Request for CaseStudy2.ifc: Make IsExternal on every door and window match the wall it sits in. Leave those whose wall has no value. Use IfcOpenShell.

First a look at what the model holds.

```python
import ifcopenshell
import ifcopenshell.util.element

model = ifcopenshell.open("CaseStudy2.ifc")
print(model.schema)
seen = {}
for e in model.by_type("IfcDoor") + model.by_type("IfcWindow"):
    if not e.FillsVoids:
        continue
    host = e.FillsVoids[0].RelatingOpeningElement.VoidsElements[0].RelatingBuildingElement
    own = ifcopenshell.util.element.get_pset(e, f"Pset_{e.is_a()[3:].removesuffix('StandardCase')}Common", "IsExternal")
    wall = ifcopenshell.util.element.get_pset(host, "Pset_WallCommon", "IsExternal")
    seen[e.is_a(), own, wall] = seen.get((e.is_a(), own, wall), 0) + 1
for (cls, own, wall), count in sorted(seen.items(), key=str):
    print(count, cls, "IsExternal:", own, "| host wall:", wall)
```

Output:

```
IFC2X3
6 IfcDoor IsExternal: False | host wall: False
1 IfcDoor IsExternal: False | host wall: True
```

```python
import ifcopenshell
import ifcopenshell.api.pset
import ifcopenshell.util.element

model = ifcopenshell.open("CaseStudy2.ifc")

count = 0
for ifc_class, pset_name in (("IfcDoor", "Pset_DoorCommon"), ("IfcWindow", "Pset_WindowCommon")):
    for e in model.by_type(ifc_class):
        if not e.FillsVoids:
            continue
        host = e.FillsVoids[0].RelatingOpeningElement.VoidsElements[0].RelatingBuildingElement
        external = ifcopenshell.util.element.get_pset(host, "Pset_WallCommon", "IsExternal")
        if external is None or ifcopenshell.util.element.get_pset(e, pset_name, "IsExternal") == external:
            continue
        pset = ifcopenshell.api.pset.add_pset(model, product=e, name=pset_name)
        ifcopenshell.api.pset.edit_pset(model, pset=pset, properties={"IsExternal": external})
        count += 1

print(count, "updated")

model.write("CaseStudy2-out.ifc")
```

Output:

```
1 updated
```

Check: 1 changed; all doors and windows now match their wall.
